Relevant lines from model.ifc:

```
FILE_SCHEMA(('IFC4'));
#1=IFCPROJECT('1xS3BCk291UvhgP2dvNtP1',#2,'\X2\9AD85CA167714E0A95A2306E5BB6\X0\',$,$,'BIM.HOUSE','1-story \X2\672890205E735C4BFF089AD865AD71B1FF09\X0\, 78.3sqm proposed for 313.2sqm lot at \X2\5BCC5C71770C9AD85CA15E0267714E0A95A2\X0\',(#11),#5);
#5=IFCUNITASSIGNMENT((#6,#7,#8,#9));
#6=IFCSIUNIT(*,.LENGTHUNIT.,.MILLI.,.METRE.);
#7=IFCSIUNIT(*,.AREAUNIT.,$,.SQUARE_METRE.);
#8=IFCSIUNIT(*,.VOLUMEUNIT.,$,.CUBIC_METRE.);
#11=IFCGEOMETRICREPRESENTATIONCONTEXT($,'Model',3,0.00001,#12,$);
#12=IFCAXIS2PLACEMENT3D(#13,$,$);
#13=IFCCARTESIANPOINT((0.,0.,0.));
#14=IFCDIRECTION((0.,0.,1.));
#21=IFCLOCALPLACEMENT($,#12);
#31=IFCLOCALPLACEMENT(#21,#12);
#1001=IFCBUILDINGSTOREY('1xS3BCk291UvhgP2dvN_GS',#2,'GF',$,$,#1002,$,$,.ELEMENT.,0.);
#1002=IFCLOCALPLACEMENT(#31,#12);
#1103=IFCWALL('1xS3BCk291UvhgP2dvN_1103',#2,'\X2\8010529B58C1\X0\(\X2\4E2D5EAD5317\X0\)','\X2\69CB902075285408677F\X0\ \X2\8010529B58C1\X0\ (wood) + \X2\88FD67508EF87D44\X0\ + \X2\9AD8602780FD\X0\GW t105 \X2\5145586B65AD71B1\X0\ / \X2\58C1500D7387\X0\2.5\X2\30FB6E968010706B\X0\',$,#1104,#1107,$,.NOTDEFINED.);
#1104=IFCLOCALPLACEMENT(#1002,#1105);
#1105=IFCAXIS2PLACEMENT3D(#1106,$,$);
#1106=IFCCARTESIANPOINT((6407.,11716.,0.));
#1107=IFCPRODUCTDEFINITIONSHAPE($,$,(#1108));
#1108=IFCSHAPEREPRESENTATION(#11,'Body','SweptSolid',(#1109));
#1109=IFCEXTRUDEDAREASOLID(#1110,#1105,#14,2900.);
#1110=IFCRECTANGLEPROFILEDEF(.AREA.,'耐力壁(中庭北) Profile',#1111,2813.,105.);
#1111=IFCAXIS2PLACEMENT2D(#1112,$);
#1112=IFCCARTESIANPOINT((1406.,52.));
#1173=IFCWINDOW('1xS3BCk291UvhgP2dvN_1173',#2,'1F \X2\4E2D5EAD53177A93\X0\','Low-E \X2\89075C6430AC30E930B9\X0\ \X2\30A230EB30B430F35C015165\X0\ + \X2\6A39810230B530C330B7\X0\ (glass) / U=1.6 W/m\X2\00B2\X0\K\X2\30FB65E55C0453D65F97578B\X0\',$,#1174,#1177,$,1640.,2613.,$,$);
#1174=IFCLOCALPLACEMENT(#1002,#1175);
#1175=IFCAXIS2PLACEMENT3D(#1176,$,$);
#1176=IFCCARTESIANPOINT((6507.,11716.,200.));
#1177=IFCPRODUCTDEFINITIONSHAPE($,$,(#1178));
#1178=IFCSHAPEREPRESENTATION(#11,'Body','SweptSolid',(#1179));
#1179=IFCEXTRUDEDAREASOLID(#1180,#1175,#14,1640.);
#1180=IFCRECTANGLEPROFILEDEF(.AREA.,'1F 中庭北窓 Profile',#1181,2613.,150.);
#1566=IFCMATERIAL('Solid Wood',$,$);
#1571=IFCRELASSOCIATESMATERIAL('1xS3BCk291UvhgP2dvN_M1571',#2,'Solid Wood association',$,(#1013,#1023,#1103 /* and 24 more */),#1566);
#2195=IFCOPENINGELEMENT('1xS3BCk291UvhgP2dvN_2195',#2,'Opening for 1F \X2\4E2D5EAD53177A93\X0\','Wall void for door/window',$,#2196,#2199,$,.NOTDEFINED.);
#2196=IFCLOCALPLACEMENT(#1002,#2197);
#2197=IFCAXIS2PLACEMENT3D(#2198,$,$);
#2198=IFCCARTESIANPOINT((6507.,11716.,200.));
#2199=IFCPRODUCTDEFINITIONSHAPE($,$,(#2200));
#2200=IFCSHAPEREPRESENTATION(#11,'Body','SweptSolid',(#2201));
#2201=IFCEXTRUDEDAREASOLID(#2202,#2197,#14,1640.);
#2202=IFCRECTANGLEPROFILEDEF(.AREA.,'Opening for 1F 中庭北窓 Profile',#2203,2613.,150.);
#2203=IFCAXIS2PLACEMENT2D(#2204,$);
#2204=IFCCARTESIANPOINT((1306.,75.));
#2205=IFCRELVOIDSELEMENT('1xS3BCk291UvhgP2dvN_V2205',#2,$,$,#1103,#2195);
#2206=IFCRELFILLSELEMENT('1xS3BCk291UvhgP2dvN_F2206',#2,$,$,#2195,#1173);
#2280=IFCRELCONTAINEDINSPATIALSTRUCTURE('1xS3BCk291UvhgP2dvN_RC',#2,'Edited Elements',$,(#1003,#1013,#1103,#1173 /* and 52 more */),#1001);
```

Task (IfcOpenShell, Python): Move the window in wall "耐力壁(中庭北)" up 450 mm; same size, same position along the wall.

```python
import numpy as np
import ifcopenshell
import ifcopenshell.api.geometry
import ifcopenshell.util.placement
import ifcopenshell.util.unit

model = ifcopenshell.open("model.ifc")
unit_scale = ifcopenshell.util.unit.calculate_unit_scale(model)

window = model.by_id(1173)
opening = window.FillsVoids[0].RelatingOpeningElement
dz = 450.0

shift = np.array([0.0, 0.0, dz])
# The window is not placed relative to its opening, so move both.
for product in (opening, window):
    matrix = ifcopenshell.util.placement.get_local_placement(product.ObjectPlacement)
    matrix[:3, 3] += shift
    ifcopenshell.api.geometry.edit_object_placement(model, product=product, matrix=matrix, is_si=False)

print(f"moved by {dz * unit_scale:+.3f} m")

model.write("model_v2.ifc")
```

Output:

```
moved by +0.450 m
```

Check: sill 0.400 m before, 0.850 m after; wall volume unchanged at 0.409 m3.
